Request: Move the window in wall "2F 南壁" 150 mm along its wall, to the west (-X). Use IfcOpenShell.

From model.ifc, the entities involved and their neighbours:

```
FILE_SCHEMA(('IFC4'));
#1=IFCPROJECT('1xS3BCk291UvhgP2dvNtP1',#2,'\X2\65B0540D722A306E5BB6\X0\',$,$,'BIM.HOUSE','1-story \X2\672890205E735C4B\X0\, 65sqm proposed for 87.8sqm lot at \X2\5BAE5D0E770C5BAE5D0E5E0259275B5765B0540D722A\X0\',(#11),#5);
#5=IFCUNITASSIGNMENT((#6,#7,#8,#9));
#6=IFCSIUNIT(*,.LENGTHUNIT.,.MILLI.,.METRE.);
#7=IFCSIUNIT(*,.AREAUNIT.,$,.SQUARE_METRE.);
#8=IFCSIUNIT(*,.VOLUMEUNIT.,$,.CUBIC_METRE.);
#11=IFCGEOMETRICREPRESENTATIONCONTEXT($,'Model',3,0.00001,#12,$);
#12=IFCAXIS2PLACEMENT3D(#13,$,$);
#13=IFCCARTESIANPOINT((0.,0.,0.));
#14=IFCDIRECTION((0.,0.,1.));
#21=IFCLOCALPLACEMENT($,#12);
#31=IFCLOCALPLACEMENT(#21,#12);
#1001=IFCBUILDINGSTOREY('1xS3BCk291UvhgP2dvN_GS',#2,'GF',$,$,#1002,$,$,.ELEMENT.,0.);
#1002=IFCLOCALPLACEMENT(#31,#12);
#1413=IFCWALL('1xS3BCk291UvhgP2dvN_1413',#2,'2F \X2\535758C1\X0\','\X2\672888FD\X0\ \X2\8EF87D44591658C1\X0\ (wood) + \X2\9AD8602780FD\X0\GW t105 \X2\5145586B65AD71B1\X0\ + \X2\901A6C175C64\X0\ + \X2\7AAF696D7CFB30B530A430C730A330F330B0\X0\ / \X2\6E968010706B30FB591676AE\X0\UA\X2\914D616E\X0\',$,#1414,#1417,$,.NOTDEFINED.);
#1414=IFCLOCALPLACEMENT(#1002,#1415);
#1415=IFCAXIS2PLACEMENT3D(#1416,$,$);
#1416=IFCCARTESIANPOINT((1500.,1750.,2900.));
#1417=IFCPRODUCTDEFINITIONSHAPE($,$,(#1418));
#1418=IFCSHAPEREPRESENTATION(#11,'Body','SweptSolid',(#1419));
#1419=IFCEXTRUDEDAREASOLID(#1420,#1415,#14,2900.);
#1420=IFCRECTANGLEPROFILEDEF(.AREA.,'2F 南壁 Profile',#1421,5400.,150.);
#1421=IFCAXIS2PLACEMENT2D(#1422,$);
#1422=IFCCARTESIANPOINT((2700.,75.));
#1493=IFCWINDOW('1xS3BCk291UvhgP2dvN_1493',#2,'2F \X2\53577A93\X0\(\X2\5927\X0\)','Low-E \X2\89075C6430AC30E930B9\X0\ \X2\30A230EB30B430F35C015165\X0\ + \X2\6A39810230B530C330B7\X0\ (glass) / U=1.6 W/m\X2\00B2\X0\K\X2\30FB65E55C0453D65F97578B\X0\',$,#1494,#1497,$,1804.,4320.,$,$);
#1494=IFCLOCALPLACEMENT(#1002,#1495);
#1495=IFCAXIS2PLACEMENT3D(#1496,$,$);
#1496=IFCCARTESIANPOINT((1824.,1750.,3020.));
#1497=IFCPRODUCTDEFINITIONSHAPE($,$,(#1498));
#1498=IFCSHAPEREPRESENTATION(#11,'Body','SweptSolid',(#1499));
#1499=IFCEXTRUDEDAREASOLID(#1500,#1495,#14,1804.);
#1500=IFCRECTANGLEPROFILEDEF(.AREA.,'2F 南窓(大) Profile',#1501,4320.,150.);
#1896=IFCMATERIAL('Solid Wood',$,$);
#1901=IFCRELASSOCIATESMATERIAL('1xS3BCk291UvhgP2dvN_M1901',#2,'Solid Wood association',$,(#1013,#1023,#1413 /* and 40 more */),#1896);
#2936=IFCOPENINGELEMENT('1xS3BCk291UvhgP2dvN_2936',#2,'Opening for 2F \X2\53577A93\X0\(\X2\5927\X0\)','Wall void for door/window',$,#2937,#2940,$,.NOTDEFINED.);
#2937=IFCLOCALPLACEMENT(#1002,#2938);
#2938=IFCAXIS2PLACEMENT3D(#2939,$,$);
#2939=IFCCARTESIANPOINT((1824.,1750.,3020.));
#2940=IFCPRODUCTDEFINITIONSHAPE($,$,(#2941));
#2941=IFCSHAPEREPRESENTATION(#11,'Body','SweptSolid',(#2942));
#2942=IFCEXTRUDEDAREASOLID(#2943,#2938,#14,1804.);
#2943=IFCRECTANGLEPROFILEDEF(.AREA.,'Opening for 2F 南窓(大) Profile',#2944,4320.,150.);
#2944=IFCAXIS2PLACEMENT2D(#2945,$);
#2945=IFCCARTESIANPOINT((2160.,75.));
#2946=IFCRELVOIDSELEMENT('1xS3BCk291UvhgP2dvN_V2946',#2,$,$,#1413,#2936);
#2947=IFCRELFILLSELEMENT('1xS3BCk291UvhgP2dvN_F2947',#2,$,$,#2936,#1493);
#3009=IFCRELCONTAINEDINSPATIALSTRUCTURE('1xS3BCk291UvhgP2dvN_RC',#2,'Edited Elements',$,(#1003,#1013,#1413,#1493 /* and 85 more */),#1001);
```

```python
import ifcopenshell
import ifcopenshell.api.geometry
import ifcopenshell.util.placement

model = ifcopenshell.open("model.ifc")

window = model.by_guid("1xS3BCk291UvhgP2dvN_1493")
opening = window.FillsVoids[0].RelatingOpeningElement
wall = opening.VoidsElements[0].RelatingBuildingElement

wall_matrix = ifcopenshell.util.placement.get_local_placement(wall.ObjectPlacement)
shift = wall_matrix[:3, 0] * -150.0
before = ifcopenshell.util.placement.get_local_placement(window.ObjectPlacement)[:3, 3].copy()

# The window is not placed relative to its opening, so move both.
for product in (opening, window):
    matrix = ifcopenshell.util.placement.get_local_placement(product.ObjectPlacement)
    matrix[:3, 3] += shift
    ifcopenshell.api.geometry.edit_object_placement(model, product=product, matrix=matrix, is_si=False)

after = ifcopenshell.util.placement.get_local_placement(window.ObjectPlacement)[:3, 3]
print("window moved by", (after - before).round(3) + 0.0)

model.write("model_v2.ifc")
```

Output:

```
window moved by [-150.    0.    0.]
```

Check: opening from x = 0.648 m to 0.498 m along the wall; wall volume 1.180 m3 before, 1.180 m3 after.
